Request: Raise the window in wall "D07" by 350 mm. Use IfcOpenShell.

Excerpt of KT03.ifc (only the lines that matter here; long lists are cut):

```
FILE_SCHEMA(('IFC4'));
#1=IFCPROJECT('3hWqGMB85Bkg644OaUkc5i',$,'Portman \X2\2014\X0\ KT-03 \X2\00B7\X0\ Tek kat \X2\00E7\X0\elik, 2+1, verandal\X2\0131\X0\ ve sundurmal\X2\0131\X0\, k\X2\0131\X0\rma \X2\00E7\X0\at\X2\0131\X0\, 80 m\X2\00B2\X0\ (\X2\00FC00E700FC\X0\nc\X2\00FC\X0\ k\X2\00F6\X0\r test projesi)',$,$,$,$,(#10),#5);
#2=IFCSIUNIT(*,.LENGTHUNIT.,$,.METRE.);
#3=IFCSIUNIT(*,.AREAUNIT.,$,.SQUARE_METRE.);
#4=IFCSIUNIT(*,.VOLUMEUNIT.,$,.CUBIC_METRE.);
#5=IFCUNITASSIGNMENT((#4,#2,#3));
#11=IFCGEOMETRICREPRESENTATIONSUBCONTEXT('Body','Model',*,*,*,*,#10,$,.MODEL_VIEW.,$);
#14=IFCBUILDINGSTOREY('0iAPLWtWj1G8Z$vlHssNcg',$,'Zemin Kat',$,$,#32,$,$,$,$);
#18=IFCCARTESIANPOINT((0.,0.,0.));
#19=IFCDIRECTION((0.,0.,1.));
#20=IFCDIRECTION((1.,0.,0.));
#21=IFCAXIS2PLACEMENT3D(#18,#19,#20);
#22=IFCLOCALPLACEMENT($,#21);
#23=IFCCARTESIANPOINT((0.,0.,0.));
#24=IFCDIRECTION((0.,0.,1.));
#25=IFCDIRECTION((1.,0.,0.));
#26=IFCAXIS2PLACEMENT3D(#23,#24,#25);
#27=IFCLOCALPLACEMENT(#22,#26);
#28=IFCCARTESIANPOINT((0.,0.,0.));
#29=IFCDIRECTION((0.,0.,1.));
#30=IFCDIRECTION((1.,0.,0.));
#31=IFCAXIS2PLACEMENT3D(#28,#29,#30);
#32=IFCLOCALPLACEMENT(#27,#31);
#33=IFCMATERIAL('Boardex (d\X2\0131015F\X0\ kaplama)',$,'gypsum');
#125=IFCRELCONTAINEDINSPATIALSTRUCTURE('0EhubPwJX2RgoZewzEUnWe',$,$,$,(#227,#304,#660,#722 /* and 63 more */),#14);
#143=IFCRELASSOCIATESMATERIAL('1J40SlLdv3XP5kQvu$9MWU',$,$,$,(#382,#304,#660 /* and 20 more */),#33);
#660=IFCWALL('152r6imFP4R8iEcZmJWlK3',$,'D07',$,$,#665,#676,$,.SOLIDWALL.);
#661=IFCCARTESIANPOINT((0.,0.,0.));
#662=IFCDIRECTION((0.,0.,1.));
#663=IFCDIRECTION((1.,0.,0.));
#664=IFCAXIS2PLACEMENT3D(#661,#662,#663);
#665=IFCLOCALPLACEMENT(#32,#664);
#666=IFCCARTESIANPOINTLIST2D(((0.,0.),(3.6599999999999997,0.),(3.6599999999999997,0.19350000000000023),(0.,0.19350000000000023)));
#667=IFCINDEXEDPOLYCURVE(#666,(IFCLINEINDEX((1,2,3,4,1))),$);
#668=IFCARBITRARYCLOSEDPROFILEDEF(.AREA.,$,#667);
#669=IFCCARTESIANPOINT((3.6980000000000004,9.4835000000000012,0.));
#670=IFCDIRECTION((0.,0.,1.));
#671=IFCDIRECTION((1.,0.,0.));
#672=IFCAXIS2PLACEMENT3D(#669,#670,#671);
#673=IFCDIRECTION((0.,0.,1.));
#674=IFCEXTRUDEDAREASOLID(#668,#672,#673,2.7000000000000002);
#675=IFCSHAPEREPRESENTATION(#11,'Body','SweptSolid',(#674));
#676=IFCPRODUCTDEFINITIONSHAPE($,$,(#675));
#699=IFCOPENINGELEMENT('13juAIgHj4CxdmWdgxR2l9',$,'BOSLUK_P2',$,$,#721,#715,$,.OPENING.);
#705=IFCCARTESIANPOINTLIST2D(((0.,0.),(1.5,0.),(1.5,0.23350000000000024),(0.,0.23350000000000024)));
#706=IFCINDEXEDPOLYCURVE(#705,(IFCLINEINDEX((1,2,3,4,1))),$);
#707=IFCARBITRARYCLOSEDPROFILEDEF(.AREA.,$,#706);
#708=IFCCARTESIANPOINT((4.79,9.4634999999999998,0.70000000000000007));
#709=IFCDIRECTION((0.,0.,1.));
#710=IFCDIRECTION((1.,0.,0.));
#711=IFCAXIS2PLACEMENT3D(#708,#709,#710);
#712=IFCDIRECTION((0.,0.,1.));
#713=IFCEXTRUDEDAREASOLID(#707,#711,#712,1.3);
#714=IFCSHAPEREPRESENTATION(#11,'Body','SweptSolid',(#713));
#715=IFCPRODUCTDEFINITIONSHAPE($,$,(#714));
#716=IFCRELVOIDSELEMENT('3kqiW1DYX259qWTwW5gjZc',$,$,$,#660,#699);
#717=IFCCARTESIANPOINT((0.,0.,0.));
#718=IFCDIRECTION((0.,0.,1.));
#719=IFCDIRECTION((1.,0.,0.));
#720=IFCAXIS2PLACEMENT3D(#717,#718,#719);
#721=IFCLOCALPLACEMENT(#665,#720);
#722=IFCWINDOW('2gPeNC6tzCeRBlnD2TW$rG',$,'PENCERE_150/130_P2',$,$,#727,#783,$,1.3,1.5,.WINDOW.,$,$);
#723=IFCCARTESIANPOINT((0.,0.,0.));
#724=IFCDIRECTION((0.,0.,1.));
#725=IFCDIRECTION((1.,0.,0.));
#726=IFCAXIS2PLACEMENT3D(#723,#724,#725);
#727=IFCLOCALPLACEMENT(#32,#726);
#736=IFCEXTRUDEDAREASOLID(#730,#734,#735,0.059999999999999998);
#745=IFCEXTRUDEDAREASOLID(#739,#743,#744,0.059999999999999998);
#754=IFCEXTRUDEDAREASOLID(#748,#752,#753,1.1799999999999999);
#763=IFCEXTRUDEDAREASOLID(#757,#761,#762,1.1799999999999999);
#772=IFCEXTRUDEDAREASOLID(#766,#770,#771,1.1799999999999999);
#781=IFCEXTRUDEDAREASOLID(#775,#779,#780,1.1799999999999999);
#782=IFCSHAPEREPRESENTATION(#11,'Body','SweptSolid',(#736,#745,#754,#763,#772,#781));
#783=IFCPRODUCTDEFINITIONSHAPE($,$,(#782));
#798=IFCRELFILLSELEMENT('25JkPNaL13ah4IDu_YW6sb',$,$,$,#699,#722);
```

```python
import numpy as np
import ifcopenshell
import ifcopenshell.api.geometry
import ifcopenshell.util.placement
import ifcopenshell.util.unit

model = ifcopenshell.open("KT03.ifc")
unit_scale = ifcopenshell.util.unit.calculate_unit_scale(model)

window = model.by_id(722)
opening = window.FillsVoids[0].RelatingOpeningElement
dz = 0.35

shift = np.array([0.0, 0.0, dz])
# The window is not placed relative to its opening, so move both.
for product in (opening, window):
    matrix = ifcopenshell.util.placement.get_local_placement(product.ObjectPlacement)
    matrix[:3, 3] += shift
    ifcopenshell.api.geometry.edit_object_placement(model, product=product, matrix=matrix, is_si=False)

print(f"moved by {dz * unit_scale:+.3f} m")

model.write("KT03_updated.ifc")
```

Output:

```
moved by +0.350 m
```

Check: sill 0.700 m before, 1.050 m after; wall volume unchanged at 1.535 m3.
